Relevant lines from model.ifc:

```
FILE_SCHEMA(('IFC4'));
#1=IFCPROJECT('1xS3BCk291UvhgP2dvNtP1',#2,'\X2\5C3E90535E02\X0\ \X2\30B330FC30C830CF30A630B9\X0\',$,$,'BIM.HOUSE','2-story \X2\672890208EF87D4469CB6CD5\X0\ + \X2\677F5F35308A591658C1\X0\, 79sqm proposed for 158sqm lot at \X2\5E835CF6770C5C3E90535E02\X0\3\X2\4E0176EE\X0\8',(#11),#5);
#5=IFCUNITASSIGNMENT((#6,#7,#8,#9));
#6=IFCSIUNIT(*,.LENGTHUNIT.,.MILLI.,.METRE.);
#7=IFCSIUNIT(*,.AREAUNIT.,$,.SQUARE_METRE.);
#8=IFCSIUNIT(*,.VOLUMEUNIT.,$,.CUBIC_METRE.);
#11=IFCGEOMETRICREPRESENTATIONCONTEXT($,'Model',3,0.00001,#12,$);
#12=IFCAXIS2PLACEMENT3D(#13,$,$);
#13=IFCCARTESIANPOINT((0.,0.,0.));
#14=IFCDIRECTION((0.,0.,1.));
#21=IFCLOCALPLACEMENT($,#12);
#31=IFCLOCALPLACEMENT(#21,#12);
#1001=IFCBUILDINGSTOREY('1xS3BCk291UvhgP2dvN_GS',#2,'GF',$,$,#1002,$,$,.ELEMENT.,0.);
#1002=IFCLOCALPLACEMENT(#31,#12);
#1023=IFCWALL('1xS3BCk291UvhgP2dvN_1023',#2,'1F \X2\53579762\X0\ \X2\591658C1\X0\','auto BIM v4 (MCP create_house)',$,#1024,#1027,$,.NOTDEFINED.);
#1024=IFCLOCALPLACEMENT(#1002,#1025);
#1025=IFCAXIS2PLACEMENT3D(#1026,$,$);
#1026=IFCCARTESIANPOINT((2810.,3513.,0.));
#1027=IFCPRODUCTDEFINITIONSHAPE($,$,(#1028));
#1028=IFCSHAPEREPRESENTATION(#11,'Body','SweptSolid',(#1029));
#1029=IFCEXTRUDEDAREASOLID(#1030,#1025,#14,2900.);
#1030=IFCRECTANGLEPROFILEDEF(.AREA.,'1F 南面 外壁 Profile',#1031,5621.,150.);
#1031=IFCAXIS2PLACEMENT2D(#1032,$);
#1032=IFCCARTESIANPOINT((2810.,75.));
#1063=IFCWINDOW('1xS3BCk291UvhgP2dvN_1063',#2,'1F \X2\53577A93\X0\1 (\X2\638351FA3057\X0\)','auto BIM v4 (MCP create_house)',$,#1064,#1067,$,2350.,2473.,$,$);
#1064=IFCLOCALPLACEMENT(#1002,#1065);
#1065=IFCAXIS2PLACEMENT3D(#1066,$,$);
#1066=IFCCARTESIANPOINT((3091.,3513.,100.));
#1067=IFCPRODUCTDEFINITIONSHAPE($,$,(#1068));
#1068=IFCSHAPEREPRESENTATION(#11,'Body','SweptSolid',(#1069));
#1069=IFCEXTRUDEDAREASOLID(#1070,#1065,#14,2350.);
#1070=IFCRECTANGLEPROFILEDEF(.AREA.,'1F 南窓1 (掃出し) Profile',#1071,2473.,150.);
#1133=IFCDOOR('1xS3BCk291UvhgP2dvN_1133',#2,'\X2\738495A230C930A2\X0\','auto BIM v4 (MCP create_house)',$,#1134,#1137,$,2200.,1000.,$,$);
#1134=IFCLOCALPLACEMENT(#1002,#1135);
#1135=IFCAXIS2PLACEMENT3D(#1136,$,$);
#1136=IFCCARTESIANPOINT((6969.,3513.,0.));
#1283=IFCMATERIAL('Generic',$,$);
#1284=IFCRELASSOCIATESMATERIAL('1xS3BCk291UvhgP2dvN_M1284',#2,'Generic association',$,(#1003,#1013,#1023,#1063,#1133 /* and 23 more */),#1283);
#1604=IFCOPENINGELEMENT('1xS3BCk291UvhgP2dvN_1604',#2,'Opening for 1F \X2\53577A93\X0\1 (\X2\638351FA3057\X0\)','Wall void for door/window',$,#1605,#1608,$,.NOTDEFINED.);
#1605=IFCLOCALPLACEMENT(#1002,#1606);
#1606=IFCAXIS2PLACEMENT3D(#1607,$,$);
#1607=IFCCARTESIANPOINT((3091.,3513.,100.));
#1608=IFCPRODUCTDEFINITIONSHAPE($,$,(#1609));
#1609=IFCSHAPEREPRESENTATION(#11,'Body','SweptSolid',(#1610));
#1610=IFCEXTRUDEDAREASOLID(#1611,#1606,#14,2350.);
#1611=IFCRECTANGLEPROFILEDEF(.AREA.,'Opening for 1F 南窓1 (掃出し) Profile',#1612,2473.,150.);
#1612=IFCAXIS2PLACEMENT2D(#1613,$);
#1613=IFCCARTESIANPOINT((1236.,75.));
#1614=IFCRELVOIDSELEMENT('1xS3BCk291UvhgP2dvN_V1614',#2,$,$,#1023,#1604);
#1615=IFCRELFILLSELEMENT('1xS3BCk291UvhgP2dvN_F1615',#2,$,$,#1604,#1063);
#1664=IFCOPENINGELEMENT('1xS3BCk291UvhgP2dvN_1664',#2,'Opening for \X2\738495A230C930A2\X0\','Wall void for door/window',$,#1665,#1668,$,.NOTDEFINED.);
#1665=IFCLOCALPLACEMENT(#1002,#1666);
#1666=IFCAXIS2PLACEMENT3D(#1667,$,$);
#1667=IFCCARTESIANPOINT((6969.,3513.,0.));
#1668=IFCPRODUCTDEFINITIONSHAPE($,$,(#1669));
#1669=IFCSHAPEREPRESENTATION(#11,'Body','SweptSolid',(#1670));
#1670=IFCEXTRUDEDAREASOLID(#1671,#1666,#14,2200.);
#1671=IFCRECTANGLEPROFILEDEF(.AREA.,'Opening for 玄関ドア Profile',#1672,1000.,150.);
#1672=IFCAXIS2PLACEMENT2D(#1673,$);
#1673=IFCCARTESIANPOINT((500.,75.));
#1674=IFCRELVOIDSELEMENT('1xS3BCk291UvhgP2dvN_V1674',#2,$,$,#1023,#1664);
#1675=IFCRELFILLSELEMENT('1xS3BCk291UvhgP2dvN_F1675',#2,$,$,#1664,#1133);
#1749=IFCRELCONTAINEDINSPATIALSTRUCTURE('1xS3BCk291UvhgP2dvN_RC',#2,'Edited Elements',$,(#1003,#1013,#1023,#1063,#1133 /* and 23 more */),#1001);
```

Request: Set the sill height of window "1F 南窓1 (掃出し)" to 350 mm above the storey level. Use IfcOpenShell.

```python
import numpy as np
import ifcopenshell
import ifcopenshell.api.geometry
import ifcopenshell.geom
import ifcopenshell.util.element
import ifcopenshell.util.placement
import ifcopenshell.util.shape
import ifcopenshell.util.unit

model = ifcopenshell.open("model.ifc")
unit_scale = ifcopenshell.util.unit.calculate_unit_scale(model)

window = model.by_guid("1xS3BCk291UvhgP2dvN_1063")
opening = window.FillsVoids[0].RelatingOpeningElement
storey = ifcopenshell.util.element.get_container(window, ifc_class="IfcBuildingStorey")
level = ifcopenshell.util.placement.get_local_placement(storey.ObjectPlacement)[2, 3]

# The opening's origin need not be at the sill, so measure its lowest point.
shape = ifcopenshell.geom.create_shape(ifcopenshell.geom.settings(), opening)
bottom = ifcopenshell.util.shape.get_shape_bottom_elevation(shape, shape.geometry) / unit_scale
dz = level + 0.35 / unit_scale - bottom

shift = np.array([0.0, 0.0, dz])
# The window is not placed relative to its opening, so move both.
for product in (opening, window):
    matrix = ifcopenshell.util.placement.get_local_placement(product.ObjectPlacement)
    matrix[:3, 3] += shift
    ifcopenshell.api.geometry.edit_object_placement(model, product=product, matrix=matrix, is_si=False)

print(f"moved by {dz * unit_scale:+.3f} m")

model.write("model-out.ifc")
```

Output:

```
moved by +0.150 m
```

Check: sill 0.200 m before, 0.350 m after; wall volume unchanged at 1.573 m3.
